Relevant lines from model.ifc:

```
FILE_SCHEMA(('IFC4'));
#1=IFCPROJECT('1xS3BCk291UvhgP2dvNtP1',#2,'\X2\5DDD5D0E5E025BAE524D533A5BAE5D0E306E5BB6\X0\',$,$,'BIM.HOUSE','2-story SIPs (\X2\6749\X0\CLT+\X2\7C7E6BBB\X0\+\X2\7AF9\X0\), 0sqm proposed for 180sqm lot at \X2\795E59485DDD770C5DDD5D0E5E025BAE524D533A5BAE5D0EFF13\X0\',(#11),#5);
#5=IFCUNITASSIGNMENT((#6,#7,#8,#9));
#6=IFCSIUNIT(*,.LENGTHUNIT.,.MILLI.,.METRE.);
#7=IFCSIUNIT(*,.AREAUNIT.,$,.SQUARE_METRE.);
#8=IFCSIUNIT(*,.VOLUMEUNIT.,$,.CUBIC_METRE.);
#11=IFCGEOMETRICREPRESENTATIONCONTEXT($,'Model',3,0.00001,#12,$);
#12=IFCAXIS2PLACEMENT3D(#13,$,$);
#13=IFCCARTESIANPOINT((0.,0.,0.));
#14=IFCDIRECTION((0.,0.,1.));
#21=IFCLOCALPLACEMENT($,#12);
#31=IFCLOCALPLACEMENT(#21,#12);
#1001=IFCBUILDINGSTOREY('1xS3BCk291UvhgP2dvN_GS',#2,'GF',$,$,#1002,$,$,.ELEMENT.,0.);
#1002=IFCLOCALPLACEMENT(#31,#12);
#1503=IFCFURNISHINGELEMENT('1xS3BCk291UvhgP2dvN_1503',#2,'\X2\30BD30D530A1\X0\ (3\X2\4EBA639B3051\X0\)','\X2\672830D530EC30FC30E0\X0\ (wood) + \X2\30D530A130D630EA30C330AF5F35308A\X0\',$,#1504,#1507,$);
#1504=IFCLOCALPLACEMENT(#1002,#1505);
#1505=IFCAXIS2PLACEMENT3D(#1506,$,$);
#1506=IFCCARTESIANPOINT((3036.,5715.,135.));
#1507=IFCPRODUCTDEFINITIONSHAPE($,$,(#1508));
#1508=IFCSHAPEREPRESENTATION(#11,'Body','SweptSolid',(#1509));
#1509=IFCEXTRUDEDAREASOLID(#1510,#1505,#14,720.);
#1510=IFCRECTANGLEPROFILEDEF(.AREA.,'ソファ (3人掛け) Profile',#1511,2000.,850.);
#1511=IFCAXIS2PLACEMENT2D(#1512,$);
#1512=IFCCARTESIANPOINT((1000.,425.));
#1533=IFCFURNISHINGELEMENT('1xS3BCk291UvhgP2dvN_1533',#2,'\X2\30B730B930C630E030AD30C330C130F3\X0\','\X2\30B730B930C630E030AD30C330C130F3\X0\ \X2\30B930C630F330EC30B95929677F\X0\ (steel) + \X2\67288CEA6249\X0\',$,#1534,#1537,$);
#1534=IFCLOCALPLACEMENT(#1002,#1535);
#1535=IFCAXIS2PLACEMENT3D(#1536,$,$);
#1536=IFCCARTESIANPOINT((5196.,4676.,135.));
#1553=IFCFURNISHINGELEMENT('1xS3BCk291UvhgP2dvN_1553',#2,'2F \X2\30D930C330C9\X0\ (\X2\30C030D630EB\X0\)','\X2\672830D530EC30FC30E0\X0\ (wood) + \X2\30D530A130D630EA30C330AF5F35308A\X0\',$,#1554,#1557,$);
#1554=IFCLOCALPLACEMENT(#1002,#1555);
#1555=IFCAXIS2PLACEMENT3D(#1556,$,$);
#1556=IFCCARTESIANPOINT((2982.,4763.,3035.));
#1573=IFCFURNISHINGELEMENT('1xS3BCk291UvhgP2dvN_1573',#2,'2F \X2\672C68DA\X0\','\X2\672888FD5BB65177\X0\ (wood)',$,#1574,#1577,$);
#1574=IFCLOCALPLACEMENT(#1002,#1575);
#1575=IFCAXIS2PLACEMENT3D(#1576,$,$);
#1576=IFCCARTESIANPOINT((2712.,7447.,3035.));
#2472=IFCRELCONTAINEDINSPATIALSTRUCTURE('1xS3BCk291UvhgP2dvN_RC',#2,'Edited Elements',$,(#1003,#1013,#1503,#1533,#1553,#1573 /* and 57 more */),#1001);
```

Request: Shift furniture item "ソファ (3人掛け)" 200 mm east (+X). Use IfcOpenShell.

```python
import ifcopenshell
import ifcopenshell.api.geometry
import ifcopenshell.util.placement
import ifcopenshell.util.unit

model = ifcopenshell.open("model.ifc")
unit_scale = ifcopenshell.util.unit.calculate_unit_scale(model)

item = model.by_guid("1xS3BCk291UvhgP2dvN_1503")
matrix = ifcopenshell.util.placement.get_local_placement(item.ObjectPlacement)
matrix[0, 3] += 0.2 / unit_scale
ifcopenshell.api.geometry.edit_object_placement(model, product=item, matrix=matrix, is_si=False)

print(ifcopenshell.util.placement.get_local_placement(item.ObjectPlacement).round(3) + 0.0)

model.write("model_rev.ifc")
```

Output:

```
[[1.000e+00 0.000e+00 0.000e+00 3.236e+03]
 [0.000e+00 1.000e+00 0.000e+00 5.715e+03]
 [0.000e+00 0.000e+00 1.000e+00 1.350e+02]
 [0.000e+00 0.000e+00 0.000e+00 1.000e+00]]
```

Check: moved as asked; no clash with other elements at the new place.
